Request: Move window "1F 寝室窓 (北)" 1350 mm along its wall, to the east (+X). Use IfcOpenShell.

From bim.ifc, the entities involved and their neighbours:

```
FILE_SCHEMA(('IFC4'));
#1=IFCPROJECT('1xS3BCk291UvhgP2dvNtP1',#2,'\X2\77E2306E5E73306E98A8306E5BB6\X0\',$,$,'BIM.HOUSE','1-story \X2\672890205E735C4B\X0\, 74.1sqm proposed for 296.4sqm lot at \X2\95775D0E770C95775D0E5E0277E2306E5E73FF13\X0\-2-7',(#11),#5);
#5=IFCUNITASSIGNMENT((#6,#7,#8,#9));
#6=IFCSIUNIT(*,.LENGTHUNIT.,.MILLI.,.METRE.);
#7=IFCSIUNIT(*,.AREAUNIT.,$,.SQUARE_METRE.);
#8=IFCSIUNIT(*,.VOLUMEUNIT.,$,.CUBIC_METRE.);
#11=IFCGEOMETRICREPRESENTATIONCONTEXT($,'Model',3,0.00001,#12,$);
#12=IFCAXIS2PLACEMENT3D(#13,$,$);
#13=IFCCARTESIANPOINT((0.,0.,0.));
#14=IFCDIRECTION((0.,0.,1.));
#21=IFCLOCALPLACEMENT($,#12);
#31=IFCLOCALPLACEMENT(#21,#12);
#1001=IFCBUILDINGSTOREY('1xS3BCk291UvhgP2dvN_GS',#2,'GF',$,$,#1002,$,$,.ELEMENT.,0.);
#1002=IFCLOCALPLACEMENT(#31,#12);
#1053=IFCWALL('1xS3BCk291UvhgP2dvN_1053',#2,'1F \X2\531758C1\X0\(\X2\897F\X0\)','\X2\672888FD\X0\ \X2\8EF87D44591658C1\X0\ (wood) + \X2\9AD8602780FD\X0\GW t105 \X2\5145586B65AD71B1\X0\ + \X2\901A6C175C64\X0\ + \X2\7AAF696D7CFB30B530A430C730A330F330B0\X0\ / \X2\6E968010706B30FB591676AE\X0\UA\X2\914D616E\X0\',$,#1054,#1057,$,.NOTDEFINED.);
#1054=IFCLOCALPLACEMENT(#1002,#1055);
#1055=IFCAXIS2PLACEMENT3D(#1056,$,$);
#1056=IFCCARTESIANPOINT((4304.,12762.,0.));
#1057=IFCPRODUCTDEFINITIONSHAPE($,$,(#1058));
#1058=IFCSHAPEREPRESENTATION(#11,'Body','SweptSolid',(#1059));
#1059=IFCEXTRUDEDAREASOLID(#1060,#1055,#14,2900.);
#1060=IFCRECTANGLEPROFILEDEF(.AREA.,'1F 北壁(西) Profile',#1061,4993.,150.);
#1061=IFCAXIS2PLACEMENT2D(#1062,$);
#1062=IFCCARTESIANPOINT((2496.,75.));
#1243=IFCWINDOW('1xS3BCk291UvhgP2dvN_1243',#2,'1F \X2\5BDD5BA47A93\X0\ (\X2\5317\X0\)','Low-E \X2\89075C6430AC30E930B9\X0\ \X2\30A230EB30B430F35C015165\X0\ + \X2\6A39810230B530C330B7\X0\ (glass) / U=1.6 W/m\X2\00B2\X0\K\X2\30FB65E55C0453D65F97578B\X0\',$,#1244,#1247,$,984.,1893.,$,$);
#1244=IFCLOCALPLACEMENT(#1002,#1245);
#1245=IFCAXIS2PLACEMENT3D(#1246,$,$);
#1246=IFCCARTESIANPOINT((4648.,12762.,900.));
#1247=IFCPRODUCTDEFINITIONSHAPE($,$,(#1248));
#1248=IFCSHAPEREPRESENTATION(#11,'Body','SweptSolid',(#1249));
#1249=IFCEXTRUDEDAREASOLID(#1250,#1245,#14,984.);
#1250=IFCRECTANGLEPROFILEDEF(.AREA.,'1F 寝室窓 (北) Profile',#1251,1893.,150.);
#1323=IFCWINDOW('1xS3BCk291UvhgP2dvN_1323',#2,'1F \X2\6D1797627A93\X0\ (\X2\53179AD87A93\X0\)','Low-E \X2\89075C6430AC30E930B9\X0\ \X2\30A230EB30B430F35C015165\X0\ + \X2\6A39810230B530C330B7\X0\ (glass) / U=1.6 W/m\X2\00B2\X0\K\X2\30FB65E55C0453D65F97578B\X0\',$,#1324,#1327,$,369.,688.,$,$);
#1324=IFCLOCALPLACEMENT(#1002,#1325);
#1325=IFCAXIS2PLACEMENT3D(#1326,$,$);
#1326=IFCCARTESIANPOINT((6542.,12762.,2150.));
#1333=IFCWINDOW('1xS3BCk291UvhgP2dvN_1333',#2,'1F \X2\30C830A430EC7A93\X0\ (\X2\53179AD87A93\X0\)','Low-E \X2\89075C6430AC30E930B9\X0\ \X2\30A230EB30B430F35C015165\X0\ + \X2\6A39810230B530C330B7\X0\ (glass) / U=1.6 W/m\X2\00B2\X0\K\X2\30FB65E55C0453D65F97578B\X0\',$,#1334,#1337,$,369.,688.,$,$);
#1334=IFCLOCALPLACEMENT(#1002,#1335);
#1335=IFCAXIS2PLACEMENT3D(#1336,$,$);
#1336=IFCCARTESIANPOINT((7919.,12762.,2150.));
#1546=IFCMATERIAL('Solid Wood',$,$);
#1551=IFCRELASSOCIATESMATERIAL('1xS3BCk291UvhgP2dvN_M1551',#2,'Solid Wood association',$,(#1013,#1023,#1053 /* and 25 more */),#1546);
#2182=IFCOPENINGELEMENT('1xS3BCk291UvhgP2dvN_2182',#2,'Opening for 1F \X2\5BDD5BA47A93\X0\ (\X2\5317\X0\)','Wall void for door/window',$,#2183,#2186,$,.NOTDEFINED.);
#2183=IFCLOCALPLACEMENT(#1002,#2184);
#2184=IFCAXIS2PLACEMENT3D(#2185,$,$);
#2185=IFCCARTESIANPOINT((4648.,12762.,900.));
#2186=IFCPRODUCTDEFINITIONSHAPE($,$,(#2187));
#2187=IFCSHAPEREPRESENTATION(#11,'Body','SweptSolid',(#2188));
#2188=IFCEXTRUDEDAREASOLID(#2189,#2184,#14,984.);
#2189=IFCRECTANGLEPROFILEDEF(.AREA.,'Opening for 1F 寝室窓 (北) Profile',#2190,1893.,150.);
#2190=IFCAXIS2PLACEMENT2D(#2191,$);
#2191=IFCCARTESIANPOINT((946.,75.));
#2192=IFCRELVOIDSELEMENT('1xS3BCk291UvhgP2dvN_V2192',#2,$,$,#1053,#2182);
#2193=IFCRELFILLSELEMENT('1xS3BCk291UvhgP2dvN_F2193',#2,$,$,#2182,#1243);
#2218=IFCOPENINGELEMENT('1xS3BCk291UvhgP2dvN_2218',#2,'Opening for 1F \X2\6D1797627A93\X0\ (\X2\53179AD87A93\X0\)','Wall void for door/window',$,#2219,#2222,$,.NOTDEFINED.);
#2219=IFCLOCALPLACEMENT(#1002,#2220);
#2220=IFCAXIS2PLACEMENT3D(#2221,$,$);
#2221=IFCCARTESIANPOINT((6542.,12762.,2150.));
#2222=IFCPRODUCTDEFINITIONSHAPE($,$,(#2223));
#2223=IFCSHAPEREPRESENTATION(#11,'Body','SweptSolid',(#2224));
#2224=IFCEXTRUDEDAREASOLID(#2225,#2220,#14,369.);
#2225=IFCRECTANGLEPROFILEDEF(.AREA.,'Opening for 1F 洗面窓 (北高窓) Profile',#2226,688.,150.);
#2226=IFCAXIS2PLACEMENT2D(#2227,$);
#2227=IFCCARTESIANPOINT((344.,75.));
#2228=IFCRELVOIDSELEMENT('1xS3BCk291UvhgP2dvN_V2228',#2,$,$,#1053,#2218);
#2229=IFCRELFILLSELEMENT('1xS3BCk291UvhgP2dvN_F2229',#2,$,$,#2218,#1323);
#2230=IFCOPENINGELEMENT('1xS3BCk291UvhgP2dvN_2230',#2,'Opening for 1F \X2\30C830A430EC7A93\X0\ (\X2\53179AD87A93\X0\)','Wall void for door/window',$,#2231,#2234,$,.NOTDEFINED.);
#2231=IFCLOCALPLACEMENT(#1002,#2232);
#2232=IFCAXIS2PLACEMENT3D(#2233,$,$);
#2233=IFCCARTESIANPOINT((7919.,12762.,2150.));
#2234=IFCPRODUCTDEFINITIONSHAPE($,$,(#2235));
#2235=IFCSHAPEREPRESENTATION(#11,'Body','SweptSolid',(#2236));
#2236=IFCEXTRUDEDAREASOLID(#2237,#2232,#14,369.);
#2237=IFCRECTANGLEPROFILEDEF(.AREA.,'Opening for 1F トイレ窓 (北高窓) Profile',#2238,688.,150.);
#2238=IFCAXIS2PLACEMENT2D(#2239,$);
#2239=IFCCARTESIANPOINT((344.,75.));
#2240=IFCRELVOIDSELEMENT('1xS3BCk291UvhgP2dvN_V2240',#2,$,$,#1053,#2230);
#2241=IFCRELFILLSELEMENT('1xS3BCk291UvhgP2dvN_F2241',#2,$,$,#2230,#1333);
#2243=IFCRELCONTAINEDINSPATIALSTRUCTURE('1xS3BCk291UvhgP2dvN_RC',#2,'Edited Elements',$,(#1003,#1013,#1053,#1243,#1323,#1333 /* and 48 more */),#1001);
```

```python
import ifcopenshell
import ifcopenshell.api.geometry
import ifcopenshell.util.placement
import ifcopenshell.util.unit

model = ifcopenshell.open("bim.ifc")
unit_scale = ifcopenshell.util.unit.calculate_unit_scale(model)

window = model.by_guid("1xS3BCk291UvhgP2dvN_1243")
opening = window.FillsVoids[0].RelatingOpeningElement
wall = opening.VoidsElements[0].RelatingBuildingElement

wall_matrix = ifcopenshell.util.placement.get_local_placement(wall.ObjectPlacement)
shift = wall_matrix[:3, 0] * 1.35 / unit_scale
before = ifcopenshell.util.placement.get_local_placement(window.ObjectPlacement)[:3, 3].copy()

# The window is not placed relative to its opening, so move both.
for product in (opening, window):
    matrix = ifcopenshell.util.placement.get_local_placement(product.ObjectPlacement)
    matrix[:3, 3] += shift
    ifcopenshell.api.geometry.edit_object_placement(model, product=product, matrix=matrix, is_si=False)

after = ifcopenshell.util.placement.get_local_placement(window.ObjectPlacement)[:3, 3]
print("window moved by", (after - before).round(3) + 0.0)

model.write("bim-out.ifc")
```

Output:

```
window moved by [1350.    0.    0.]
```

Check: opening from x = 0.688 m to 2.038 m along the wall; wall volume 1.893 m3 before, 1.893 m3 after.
